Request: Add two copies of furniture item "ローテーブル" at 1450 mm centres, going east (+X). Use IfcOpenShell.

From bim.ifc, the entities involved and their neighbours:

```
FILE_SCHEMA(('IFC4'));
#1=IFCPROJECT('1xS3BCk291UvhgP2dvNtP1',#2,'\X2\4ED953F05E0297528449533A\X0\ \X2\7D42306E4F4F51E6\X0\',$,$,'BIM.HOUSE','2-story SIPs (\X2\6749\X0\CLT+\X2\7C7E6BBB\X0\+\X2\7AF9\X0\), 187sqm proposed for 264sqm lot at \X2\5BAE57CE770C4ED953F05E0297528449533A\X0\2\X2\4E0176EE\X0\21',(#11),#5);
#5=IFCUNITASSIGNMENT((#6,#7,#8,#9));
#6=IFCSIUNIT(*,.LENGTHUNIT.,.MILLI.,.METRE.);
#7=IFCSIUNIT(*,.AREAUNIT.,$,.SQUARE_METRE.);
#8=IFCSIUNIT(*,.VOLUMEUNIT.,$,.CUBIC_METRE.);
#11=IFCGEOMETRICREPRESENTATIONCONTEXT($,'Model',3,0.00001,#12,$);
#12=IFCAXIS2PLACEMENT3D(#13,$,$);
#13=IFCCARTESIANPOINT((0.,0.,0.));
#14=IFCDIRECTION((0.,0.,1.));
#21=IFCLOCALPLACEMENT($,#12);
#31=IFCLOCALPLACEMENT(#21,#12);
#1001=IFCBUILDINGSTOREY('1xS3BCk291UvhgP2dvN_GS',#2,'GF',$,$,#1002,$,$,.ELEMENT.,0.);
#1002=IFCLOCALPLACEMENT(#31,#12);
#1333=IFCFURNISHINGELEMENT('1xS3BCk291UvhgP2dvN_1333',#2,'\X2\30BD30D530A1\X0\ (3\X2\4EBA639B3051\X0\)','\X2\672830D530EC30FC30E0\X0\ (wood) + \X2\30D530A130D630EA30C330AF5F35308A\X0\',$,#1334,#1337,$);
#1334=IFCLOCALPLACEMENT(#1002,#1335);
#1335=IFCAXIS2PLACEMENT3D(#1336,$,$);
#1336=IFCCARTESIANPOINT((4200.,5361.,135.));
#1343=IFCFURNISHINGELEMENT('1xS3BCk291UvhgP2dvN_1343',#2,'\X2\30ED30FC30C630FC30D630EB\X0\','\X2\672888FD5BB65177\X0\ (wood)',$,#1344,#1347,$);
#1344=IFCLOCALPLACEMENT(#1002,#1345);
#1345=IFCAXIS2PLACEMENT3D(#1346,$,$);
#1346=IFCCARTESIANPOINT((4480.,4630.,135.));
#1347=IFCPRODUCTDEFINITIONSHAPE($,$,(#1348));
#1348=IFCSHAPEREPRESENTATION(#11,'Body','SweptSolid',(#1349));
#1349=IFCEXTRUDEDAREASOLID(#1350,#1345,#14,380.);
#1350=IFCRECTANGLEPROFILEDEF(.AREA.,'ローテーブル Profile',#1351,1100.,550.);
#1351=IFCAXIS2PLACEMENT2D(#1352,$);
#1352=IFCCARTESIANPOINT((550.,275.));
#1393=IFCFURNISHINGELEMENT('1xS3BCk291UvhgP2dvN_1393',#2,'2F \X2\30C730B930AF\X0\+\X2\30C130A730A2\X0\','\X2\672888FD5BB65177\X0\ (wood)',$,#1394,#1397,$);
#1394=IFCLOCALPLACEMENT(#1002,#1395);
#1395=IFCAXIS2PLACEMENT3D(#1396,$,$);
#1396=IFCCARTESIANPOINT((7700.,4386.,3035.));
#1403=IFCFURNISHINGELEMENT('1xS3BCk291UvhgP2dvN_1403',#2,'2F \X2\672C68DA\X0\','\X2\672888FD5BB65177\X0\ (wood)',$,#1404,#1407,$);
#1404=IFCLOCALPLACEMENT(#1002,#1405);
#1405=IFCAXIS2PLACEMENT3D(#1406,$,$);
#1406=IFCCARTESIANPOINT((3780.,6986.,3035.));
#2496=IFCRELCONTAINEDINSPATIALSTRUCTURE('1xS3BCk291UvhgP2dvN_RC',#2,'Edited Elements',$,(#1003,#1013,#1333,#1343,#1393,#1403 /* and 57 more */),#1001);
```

```python
import numpy as np
import ifcopenshell
import ifcopenshell.api.geometry
import ifcopenshell.api.root
import ifcopenshell.util.element
import ifcopenshell.util.placement
import ifcopenshell.util.unit

model = ifcopenshell.open("bim.ifc")
unit_scale = ifcopenshell.util.unit.calculate_unit_scale(model)


def reuse_history(source, copy):
    """copy_class also copies each property set's owner history, people and application; keep the originals."""
    for rel in copy.IsDefinedBy:
        if rel.is_a("IfcRelDefinesByProperties") and (history := rel.RelatingPropertyDefinition.OwnerHistory):
            rel.RelatingPropertyDefinition.OwnerHistory = source.OwnerHistory
            ifcopenshell.util.element.remove_deep2(model, history)


source = model.by_guid("1xS3BCk291UvhgP2dvN_1343")
base = ifcopenshell.util.placement.get_local_placement(source.ObjectPlacement)
step = np.array([1.0, 0.0, 0.0]) * 1.45 / unit_scale

for i in range(1, 3):
    copy = ifcopenshell.api.root.copy_class(model, product=source)
    copy.Representation = ifcopenshell.util.element.copy_deep(
        model, source.Representation, exclude=["IfcGeometricRepresentationContext", "IfcRepresentationMap"]
    )
    reuse_history(source, copy)
    matrix = base.copy()
    matrix[:3, 3] += i * step
    print("added at", matrix[:3, 3].round(3) + 0.0)
    ifcopenshell.api.geometry.edit_object_placement(model, product=copy, matrix=matrix, is_si=False)

model.write("bim_rev.ifc")
```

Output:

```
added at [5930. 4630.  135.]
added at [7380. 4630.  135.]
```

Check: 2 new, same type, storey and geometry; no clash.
